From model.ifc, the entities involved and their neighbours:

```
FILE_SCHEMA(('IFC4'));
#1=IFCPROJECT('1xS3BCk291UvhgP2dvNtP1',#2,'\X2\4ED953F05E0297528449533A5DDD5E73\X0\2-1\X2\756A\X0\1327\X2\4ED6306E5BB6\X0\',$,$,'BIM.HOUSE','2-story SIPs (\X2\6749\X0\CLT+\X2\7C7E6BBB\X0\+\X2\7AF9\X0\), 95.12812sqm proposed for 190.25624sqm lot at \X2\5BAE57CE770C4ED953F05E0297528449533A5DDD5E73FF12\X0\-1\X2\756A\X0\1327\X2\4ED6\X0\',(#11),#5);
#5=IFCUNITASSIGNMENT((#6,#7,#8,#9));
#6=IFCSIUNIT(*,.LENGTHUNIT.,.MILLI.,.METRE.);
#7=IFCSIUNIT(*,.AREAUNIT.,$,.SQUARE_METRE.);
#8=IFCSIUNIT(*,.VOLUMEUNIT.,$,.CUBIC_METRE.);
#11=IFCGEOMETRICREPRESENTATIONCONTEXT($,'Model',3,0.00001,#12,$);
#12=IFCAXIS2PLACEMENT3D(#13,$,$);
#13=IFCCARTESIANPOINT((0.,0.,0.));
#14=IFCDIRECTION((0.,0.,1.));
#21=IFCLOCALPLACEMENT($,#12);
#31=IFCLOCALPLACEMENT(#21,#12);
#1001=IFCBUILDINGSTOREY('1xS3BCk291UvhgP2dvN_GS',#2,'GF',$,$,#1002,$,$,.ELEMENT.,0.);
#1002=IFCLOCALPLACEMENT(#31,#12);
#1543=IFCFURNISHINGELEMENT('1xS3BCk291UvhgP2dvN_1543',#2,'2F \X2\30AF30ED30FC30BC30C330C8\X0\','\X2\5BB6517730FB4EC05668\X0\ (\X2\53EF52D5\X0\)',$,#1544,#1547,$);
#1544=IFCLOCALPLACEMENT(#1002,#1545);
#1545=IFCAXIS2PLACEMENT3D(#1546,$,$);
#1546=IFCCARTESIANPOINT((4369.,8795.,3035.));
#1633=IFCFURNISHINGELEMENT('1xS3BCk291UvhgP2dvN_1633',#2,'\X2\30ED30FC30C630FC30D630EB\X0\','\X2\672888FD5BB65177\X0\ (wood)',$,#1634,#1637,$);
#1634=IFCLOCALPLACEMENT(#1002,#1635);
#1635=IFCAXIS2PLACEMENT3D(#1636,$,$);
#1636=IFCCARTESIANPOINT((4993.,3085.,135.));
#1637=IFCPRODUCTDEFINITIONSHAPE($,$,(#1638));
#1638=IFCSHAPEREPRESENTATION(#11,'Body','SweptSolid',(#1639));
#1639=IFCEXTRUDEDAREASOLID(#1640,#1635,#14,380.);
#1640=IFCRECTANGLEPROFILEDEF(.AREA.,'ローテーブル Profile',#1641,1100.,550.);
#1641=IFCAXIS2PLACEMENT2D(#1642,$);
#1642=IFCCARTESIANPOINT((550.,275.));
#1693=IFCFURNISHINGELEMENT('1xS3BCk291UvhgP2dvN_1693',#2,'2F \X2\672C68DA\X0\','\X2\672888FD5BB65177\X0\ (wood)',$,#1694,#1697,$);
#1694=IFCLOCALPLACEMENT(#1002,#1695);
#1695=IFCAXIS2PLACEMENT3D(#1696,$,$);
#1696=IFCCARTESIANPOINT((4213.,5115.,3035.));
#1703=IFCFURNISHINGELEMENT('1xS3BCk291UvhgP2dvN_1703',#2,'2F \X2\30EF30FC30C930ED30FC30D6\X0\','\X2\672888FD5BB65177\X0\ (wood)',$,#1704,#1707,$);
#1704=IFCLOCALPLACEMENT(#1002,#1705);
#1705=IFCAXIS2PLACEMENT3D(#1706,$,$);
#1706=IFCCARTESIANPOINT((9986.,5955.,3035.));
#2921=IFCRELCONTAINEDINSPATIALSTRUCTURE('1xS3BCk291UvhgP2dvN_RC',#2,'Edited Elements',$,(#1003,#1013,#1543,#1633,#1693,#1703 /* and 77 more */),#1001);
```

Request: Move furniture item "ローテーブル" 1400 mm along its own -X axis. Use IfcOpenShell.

```python
import ifcopenshell
import ifcopenshell.api.geometry
import ifcopenshell.util.placement
import ifcopenshell.util.unit

model = ifcopenshell.open("model.ifc")
unit_scale = ifcopenshell.util.unit.calculate_unit_scale(model)

item = model.by_guid("1xS3BCk291UvhgP2dvN_1633")
matrix = ifcopenshell.util.placement.get_local_placement(item.ObjectPlacement)
matrix[:3, 3] -= matrix[:3, 0] * 1.4 / unit_scale
ifcopenshell.api.geometry.edit_object_placement(model, product=item, matrix=matrix, is_si=False)

print(ifcopenshell.util.placement.get_local_placement(item.ObjectPlacement).round(3) + 0.0)

model.write("model_edited.ifc")
```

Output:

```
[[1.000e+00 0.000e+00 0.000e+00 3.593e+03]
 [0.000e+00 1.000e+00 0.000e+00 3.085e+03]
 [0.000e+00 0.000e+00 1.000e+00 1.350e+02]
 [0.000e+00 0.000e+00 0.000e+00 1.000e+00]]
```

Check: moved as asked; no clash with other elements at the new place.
